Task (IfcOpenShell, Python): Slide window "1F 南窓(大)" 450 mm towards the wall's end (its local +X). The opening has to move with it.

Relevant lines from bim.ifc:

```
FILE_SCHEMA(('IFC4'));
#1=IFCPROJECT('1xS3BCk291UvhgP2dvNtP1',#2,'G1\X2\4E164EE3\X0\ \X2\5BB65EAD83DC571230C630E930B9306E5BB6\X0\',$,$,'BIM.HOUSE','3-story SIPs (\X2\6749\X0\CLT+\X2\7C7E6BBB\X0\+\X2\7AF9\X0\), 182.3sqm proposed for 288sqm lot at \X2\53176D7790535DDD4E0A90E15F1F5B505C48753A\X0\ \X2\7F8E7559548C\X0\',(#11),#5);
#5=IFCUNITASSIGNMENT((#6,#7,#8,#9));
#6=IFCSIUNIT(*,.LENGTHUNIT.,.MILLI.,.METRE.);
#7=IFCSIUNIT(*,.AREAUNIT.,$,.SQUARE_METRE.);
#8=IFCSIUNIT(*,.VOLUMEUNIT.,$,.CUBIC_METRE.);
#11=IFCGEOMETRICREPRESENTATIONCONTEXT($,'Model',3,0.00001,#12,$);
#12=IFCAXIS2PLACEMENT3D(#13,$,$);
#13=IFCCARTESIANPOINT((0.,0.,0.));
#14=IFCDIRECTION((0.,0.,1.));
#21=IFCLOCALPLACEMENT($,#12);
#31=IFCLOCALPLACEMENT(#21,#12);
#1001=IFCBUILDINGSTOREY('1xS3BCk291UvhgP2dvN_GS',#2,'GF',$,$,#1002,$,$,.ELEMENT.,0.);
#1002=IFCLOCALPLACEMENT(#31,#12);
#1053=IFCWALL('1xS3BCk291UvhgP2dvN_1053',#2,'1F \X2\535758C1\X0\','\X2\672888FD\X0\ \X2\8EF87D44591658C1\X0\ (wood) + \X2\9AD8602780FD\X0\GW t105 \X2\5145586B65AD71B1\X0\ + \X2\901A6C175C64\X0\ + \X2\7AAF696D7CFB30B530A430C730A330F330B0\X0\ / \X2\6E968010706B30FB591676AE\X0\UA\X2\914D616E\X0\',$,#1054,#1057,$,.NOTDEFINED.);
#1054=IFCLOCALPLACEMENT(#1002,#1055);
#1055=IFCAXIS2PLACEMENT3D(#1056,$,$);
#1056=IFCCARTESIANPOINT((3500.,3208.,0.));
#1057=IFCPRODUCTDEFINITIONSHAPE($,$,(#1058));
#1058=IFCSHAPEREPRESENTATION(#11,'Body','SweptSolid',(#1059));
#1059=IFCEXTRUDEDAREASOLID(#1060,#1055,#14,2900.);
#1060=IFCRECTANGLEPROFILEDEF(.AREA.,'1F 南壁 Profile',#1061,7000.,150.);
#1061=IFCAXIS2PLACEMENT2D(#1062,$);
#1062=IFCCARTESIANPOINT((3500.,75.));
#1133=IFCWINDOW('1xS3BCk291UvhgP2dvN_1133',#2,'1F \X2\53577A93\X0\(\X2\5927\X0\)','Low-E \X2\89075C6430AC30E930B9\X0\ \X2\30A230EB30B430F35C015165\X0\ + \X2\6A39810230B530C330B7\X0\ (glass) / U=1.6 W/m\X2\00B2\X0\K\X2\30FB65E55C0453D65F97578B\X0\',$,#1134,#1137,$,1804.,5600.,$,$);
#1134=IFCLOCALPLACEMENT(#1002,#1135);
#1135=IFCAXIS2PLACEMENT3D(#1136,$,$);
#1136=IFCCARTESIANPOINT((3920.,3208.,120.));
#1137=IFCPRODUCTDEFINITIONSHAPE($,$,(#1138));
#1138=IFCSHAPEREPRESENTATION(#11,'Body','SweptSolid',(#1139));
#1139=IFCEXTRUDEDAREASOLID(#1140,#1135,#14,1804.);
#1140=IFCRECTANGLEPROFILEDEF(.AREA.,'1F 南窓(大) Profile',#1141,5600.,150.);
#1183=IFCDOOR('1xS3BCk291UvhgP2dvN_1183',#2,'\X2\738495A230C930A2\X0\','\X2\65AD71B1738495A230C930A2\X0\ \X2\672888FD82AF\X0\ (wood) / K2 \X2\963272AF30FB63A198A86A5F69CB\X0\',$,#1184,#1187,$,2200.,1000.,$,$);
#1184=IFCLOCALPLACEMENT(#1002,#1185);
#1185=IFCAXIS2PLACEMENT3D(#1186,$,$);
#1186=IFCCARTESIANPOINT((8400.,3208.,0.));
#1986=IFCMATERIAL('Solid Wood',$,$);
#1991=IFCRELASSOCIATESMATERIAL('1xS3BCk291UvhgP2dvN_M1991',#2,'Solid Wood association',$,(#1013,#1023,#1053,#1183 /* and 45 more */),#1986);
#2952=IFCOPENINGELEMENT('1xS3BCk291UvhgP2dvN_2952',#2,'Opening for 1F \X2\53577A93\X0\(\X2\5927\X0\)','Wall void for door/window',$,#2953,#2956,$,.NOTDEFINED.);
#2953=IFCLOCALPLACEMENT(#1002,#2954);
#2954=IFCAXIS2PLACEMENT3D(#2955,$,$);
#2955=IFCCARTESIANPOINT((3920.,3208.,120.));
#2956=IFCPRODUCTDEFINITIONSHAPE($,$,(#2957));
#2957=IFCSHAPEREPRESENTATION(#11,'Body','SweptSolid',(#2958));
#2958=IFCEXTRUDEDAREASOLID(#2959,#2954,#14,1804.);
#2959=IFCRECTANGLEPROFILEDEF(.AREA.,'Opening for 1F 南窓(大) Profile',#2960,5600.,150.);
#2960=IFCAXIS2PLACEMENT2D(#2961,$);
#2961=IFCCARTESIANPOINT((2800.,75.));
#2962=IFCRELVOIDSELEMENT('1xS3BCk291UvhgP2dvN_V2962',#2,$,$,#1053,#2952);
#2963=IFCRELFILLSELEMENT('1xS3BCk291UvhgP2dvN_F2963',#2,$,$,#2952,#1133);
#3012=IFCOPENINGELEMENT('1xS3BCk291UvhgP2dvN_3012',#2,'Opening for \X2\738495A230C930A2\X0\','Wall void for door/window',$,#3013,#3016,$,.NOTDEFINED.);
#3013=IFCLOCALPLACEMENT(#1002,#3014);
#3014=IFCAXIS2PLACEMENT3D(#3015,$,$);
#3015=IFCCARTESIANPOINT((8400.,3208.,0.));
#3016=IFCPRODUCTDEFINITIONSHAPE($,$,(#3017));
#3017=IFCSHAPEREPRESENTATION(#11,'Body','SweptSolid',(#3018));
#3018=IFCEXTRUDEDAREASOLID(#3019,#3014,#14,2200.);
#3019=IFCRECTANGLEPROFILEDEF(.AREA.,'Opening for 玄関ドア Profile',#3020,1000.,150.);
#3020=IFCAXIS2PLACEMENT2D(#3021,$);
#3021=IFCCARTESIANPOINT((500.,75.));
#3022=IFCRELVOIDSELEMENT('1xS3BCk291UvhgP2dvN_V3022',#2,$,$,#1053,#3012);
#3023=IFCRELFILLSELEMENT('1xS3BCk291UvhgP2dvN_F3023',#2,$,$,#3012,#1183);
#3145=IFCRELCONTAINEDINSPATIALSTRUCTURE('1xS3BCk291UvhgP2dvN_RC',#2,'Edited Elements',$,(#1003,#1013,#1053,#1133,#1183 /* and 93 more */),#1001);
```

```python
import ifcopenshell
import ifcopenshell.api.geometry
import ifcopenshell.util.placement
import ifcopenshell.util.unit

model = ifcopenshell.open("bim.ifc")
unit_scale = ifcopenshell.util.unit.calculate_unit_scale(model)

window = model.by_id(1133)
opening = window.FillsVoids[0].RelatingOpeningElement
wall = opening.VoidsElements[0].RelatingBuildingElement

wall_matrix = ifcopenshell.util.placement.get_local_placement(wall.ObjectPlacement)
shift = wall_matrix[:3, 0] * 0.45 / unit_scale
before = ifcopenshell.util.placement.get_local_placement(window.ObjectPlacement)[:3, 3].copy()

# The window is not placed relative to its opening, so move both.
for product in (opening, window):
    matrix = ifcopenshell.util.placement.get_local_placement(product.ObjectPlacement)
    matrix[:3, 3] += shift
    ifcopenshell.api.geometry.edit_object_placement(model, product=product, matrix=matrix, is_si=False)

after = ifcopenshell.util.placement.get_local_placement(window.ObjectPlacement)[:3, 3]
print("window moved by", (after - before).round(3) + 0.0)

model.write("bim_edited.ifc")
```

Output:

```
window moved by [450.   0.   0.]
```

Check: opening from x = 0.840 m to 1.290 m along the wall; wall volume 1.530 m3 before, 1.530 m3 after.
